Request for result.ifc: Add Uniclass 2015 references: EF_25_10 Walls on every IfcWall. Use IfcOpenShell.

First a look at what the model holds.

```python
import ifcopenshell

model = ifcopenshell.open("result.ifc")
print(model.schema)
print("classifications:", [c.Name for c in model.by_type("IfcClassification")])
for ifc_class in ("IfcDoor", "IfcRoof", "IfcStair", "IfcWall", "IfcWindow"):
    print(ifc_class, len(model.by_type(ifc_class)))
```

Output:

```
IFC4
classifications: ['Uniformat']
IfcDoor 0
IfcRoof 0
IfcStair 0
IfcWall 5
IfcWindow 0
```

```python
import ifcopenshell
import ifcopenshell.api.classification

model = ifcopenshell.open("result.ifc")

system = ifcopenshell.api.classification.add_classification(model, classification="Uniclass 2015")

codes = {
    "IfcWall": ("EF_25_10", "Walls"),
}
for ifc_class, (code, name) in codes.items():
    products = model.by_type(ifc_class)
    ifcopenshell.api.classification.add_reference(
        model, products=products, classification=system, identification=code, name=name
    )
    print(code, len(products))

model.write("result_edited.ifc")
```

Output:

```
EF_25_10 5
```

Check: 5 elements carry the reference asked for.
